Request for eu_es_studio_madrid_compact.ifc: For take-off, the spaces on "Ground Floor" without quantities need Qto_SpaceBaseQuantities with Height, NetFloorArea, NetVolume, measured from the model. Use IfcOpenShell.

First a look at what the model holds.

```python
import ifcopenshell
import ifcopenshell.util.element
import ifcopenshell.util.unit

model = ifcopenshell.open("eu_es_studio_madrid_compact.ifc")
print(model.schema)
for unit_type in ("LENGTHUNIT", "AREAUNIT", "VOLUMEUNIT"):
    print(unit_type, ifcopenshell.util.unit.calculate_unit_scale(model, unit_type))
storey = next(s for s in model.by_type("IfcBuildingStorey") if s.Name == "Ground Floor")
spaces = [e for e in ifcopenshell.util.element.get_decomposition(storey) if e.is_a("IfcSpace")]
for e in sorted(spaces, key=lambda e: e.id()):
    print(e.id(), e.is_a(), e.Name, list(ifcopenshell.util.element.get_psets(e, qtos_only=True)), sep=" | ")
```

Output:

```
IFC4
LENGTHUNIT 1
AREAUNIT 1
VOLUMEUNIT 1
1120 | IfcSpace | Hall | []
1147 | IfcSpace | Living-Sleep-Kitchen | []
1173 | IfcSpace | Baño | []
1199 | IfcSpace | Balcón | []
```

```python
import ifcopenshell
import ifcopenshell.api.pset
import ifcopenshell.geom
import ifcopenshell.util.element
import ifcopenshell.util.shape
import ifcopenshell.util.unit

model = ifcopenshell.open("eu_es_studio_madrid_compact.ifc")
unit_scale = ifcopenshell.util.unit.calculate_unit_scale(model)
area_scale = ifcopenshell.util.unit.calculate_unit_scale(model, "AREAUNIT")
volume_scale = ifcopenshell.util.unit.calculate_unit_scale(model, "VOLUMEUNIT")
settings = ifcopenshell.geom.settings()

storey = next(s for s in model.by_type("IfcBuildingStorey") if s.Name == "Ground Floor")
spaces = [e for e in ifcopenshell.util.element.get_decomposition(storey) if e.is_a("IfcSpace")]

for e in sorted(spaces, key=lambda e: e.id()):
    if ifcopenshell.util.element.get_psets(e, qtos_only=True, should_inherit=False):
        continue
    # Geometry comes back in metres, in the element's own axes.
    shape = ifcopenshell.geom.create_shape(settings, e)
    values = {
        "Height": ifcopenshell.util.shape.get_z(shape.geometry) / unit_scale,
        "NetFloorArea": ifcopenshell.util.shape.get_footprint_area(shape.geometry) / area_scale,
        "NetVolume": ifcopenshell.util.shape.get_volume(shape.geometry) / volume_scale,
    }
    qto = ifcopenshell.api.pset.add_qto(model, product=e, name="Qto_SpaceBaseQuantities")
    ifcopenshell.api.pset.edit_qto(model, qto=qto, properties=values)
    print(e.id(), {k: round(v, 3) for k, v in values.items()})

model.write("eu_es_studio_madrid_compact-out.ifc")
```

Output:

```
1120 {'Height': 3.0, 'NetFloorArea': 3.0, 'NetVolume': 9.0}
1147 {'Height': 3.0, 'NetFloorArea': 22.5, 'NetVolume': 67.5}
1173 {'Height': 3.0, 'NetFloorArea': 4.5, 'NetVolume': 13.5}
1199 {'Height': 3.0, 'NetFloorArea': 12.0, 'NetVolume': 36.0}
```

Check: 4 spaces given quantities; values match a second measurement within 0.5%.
